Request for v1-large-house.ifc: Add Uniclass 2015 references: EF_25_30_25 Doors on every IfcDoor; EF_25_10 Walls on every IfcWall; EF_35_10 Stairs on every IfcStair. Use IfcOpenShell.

First a look at what the model holds.

```python
import ifcopenshell

model = ifcopenshell.open("v1-large-house.ifc")
print(model.schema)
print("classifications:", [c.Name for c in model.by_type("IfcClassification")])
for ifc_class in ("IfcDoor", "IfcRoof", "IfcStair", "IfcWall", "IfcWindow"):
    print(ifc_class, len(model.by_type(ifc_class)))
```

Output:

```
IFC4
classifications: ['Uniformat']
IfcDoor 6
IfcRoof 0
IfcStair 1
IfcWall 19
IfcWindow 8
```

```python
import ifcopenshell
import ifcopenshell.api.classification

model = ifcopenshell.open("v1-large-house.ifc")

system = ifcopenshell.api.classification.add_classification(model, classification="Uniclass 2015")

codes = {
    "IfcDoor": ("EF_25_30_25", "Doors"),
    "IfcWall": ("EF_25_10", "Walls"),
    "IfcStair": ("EF_35_10", "Stairs"),
}
for ifc_class, (code, name) in codes.items():
    products = model.by_type(ifc_class)
    ifcopenshell.api.classification.add_reference(
        model, products=products, classification=system, identification=code, name=name
    )
    print(code, len(products))

model.write("v1-large-house_v2.ifc")
```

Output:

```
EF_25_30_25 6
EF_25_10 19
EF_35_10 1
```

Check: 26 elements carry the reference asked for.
